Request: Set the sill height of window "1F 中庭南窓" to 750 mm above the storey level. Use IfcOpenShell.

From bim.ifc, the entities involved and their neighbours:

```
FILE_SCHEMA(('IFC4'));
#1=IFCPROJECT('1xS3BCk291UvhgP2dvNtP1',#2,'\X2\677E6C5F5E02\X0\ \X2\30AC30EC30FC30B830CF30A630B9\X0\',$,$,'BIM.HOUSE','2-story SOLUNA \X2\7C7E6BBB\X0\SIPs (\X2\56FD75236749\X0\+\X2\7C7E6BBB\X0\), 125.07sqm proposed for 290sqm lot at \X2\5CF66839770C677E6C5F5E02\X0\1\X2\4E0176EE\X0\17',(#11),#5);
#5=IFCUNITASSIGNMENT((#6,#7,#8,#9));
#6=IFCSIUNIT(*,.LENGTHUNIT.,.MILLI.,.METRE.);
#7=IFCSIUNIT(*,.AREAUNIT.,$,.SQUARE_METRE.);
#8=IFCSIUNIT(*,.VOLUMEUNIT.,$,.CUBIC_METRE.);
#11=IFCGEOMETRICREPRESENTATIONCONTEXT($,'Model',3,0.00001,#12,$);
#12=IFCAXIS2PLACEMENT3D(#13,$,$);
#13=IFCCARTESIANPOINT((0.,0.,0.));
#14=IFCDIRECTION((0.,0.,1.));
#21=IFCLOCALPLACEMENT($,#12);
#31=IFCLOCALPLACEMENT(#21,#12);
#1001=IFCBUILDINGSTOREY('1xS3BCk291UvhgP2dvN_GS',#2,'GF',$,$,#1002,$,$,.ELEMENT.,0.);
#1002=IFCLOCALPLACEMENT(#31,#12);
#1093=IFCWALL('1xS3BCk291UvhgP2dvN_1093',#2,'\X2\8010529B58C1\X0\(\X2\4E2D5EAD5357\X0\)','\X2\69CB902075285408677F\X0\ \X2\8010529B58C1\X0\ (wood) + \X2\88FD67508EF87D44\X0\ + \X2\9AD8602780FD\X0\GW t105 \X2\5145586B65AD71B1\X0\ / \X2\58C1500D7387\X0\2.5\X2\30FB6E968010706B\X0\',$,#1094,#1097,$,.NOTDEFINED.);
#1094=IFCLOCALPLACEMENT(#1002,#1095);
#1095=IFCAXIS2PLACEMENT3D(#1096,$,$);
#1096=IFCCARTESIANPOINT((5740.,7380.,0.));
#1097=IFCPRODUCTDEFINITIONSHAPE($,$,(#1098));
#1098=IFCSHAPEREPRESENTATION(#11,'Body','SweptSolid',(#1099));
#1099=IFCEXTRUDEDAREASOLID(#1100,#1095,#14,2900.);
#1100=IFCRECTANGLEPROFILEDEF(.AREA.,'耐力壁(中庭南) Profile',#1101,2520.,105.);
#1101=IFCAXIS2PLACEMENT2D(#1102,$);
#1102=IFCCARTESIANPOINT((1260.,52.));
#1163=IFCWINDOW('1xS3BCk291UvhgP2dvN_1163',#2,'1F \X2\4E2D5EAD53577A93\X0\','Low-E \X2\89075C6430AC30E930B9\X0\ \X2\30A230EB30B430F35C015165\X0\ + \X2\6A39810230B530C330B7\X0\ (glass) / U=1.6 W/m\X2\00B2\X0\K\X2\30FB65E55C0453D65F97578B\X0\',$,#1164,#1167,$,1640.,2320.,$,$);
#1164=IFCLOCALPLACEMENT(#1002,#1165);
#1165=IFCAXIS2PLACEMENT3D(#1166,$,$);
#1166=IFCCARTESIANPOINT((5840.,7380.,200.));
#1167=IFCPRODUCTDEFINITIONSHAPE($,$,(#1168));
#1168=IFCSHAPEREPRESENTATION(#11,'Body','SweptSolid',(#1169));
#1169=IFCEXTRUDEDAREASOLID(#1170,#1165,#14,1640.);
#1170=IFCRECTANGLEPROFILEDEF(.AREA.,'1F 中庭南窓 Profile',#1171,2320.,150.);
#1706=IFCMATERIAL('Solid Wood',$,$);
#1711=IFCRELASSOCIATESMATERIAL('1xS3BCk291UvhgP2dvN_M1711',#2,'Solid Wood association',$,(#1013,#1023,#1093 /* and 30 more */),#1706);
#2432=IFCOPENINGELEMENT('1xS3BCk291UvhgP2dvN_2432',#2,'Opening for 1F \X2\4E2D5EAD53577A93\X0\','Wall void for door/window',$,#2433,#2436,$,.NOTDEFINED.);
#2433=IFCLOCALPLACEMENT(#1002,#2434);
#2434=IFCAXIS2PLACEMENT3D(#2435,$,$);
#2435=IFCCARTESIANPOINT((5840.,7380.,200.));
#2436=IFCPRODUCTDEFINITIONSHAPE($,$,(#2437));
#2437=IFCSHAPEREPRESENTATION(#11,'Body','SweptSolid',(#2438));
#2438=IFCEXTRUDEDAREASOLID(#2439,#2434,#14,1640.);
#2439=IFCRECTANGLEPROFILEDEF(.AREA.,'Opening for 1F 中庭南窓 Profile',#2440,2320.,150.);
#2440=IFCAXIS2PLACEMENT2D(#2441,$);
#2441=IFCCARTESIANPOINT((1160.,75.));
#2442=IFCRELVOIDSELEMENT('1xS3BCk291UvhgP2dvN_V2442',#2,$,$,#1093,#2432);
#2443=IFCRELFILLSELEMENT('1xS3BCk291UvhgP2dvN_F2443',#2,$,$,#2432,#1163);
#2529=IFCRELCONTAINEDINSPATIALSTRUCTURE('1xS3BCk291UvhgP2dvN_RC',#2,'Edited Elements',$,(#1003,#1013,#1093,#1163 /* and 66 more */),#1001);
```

```python
import numpy as np
import ifcopenshell
import ifcopenshell.api.geometry
import ifcopenshell.geom
import ifcopenshell.util.element
import ifcopenshell.util.placement
import ifcopenshell.util.shape
import ifcopenshell.util.unit

model = ifcopenshell.open("bim.ifc")
unit_scale = ifcopenshell.util.unit.calculate_unit_scale(model)

window = model.by_guid("1xS3BCk291UvhgP2dvN_1163")
opening = window.FillsVoids[0].RelatingOpeningElement
storey = ifcopenshell.util.element.get_container(window, ifc_class="IfcBuildingStorey")
level = ifcopenshell.util.placement.get_local_placement(storey.ObjectPlacement)[2, 3]

# The opening's origin need not be at the sill, so measure its lowest point.
shape = ifcopenshell.geom.create_shape(ifcopenshell.geom.settings(), opening)
bottom = ifcopenshell.util.shape.get_shape_bottom_elevation(shape, shape.geometry) / unit_scale
dz = level + 0.75 / unit_scale - bottom

shift = np.array([0.0, 0.0, dz])
# The window is not placed relative to its opening, so move both.
for product in (opening, window):
    matrix = ifcopenshell.util.placement.get_local_placement(product.ObjectPlacement)
    matrix[:3, 3] += shift
    ifcopenshell.api.geometry.edit_object_placement(model, product=product, matrix=matrix, is_si=False)

print(f"moved by {dz * unit_scale:+.3f} m")

model.write("bim_updated.ifc")
```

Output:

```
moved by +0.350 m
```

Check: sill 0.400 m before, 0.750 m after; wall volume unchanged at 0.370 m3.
